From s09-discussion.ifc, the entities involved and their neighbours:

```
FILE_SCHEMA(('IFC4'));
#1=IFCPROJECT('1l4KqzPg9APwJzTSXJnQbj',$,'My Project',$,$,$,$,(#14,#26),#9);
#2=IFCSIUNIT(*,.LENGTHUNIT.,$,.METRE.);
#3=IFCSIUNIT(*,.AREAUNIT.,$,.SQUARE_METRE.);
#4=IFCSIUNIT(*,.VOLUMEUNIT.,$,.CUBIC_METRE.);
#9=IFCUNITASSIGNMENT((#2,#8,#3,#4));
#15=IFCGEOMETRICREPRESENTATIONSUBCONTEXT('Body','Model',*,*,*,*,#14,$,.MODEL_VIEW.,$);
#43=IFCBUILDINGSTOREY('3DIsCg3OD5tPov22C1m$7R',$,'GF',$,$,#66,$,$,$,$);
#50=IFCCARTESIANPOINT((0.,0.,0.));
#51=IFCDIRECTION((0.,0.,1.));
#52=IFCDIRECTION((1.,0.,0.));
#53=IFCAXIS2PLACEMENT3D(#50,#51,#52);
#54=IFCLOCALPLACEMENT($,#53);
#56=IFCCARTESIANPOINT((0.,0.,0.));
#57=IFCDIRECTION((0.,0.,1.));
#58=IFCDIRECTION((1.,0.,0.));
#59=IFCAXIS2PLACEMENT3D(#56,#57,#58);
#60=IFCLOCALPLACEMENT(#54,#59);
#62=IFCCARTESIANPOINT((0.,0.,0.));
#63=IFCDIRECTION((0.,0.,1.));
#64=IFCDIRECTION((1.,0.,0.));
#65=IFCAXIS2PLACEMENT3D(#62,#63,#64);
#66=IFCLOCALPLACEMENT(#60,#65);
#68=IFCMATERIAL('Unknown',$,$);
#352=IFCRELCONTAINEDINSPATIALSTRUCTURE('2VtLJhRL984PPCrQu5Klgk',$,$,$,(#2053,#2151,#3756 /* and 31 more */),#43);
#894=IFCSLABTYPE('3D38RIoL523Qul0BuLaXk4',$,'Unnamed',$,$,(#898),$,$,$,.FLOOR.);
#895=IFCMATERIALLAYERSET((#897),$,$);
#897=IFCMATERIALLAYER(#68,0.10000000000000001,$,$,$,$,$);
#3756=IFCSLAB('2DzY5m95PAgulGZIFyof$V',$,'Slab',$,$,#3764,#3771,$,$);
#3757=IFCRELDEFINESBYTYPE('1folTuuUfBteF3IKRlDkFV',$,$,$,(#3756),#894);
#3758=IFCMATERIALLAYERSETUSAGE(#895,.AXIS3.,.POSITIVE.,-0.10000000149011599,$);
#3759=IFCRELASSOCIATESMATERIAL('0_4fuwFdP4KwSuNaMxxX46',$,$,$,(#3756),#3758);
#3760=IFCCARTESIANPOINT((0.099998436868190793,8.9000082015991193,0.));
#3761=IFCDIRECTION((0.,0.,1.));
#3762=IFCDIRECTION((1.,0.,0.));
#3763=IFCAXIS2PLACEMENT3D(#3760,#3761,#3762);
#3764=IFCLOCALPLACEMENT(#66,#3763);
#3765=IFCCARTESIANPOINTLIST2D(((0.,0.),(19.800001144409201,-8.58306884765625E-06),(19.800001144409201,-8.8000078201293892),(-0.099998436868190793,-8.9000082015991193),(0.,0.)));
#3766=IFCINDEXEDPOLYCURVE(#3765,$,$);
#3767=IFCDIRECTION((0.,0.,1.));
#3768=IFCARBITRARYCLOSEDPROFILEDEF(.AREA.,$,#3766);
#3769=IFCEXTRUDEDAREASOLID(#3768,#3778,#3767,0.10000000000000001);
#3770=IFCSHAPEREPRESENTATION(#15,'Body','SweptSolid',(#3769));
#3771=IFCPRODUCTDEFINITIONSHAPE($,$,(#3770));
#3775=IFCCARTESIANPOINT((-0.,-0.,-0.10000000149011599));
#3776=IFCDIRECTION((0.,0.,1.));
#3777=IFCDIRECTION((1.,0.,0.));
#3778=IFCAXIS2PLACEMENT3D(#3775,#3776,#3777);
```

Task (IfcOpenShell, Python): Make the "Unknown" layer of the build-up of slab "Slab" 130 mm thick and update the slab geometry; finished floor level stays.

```python
import ifcopenshell
import ifcopenshell.util.element
import ifcopenshell.util.representation

model = ifcopenshell.open("s09-discussion.ifc")

layer_set = model.by_id(895)
layer = next(l for l in layer_set.MaterialLayers if l.Material and l.Material.Name == "Unknown")
change = 0.13 - layer.LayerThickness
layer.LayerThickness += change

# Geometry does not follow the layer set by itself.
slabs = [e for e in ifcopenshell.util.element.get_elements_by_material(model, layer_set) if e.is_a("IfcSlab")]
for slab in sorted(slabs, key=lambda e: e.id()):
    body = ifcopenshell.util.representation.get_representation(slab, "Model", "Body")
    solid = body.Items[0]
    old_depth = solid.Depth
    solid.Depth += change
    # Extruded upwards: lower the start of the extrusion so the top stays.
    x, y, z = solid.Position.Location.Coordinates
    solid.Position.Location = model.createIfcCartesianPoint((x, y, z - change))
    print(slab.id(), f"{old_depth:g} -> {solid.Depth:g}")

# The layers are counted up from the underside, which has moved.
for usage in {ifcopenshell.util.element.get_material(slab) for slab in slabs}:
    usage.OffsetFromReferenceLine -= change

model.write("s09-discussion-out.ifc")
```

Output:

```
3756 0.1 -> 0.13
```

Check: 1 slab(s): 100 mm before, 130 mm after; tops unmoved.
